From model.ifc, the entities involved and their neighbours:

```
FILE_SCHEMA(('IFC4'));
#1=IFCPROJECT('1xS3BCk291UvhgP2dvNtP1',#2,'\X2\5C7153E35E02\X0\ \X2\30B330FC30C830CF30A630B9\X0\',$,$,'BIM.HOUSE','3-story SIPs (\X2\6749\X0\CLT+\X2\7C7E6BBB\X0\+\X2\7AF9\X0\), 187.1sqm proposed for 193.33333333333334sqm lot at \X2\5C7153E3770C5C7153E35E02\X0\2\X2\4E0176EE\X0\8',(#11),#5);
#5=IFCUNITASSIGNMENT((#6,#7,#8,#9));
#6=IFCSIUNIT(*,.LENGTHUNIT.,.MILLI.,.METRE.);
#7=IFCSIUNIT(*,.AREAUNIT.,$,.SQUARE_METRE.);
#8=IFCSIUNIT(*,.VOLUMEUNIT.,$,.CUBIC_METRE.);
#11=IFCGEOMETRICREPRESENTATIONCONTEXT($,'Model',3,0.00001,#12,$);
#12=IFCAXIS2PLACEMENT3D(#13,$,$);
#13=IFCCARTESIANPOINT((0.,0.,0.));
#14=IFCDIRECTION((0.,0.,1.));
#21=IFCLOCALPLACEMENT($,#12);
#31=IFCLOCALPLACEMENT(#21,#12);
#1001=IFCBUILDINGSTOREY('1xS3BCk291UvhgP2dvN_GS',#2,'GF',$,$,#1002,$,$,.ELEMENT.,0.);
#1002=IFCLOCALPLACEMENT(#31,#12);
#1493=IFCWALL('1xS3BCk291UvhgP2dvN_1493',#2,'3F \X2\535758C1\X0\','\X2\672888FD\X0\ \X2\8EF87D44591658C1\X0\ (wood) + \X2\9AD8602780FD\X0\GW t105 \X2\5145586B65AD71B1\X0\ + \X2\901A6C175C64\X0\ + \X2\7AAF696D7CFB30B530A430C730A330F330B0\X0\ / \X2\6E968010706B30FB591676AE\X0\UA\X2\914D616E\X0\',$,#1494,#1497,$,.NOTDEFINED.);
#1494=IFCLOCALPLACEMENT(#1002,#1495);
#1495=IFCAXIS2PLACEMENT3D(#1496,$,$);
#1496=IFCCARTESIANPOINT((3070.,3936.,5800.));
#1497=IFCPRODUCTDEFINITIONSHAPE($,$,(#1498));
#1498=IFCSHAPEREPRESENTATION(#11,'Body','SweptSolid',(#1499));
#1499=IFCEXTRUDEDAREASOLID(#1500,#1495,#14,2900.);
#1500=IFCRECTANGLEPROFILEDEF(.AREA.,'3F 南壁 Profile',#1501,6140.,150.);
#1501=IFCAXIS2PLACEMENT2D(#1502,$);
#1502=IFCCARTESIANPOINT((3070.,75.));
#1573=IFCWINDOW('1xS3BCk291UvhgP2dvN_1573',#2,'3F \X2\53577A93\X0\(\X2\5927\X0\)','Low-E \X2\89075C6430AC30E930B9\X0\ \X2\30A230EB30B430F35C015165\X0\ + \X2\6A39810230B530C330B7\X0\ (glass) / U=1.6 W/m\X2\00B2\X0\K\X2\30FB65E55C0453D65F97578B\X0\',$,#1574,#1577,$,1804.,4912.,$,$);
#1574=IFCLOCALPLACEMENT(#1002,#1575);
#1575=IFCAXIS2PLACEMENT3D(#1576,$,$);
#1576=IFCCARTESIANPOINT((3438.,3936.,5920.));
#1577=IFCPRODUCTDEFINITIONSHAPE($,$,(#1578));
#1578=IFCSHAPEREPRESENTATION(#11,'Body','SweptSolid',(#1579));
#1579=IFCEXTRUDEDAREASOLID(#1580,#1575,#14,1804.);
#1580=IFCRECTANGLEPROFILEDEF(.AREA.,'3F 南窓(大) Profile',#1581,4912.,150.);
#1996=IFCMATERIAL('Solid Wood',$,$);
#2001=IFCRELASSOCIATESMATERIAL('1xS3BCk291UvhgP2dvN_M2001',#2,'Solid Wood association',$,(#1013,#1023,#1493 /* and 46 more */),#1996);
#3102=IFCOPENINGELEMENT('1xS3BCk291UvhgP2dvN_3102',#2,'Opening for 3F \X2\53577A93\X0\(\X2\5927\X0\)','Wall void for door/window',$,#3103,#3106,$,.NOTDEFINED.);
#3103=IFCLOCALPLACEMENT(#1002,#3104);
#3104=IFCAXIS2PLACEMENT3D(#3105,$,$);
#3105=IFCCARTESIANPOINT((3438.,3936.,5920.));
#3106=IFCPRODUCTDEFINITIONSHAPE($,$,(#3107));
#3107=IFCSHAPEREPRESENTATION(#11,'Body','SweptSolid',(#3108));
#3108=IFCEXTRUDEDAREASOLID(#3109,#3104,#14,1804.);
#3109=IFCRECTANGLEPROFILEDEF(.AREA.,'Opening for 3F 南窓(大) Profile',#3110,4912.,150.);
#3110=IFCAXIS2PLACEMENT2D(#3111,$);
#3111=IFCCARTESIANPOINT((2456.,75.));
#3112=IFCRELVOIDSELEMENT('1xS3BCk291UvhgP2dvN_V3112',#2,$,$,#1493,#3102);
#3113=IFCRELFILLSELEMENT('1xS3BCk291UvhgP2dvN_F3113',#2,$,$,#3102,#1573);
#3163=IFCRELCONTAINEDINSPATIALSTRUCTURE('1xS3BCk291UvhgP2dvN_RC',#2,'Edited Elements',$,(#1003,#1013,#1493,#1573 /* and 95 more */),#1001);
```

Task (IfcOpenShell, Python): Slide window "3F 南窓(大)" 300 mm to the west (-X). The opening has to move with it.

```python
import ifcopenshell
import ifcopenshell.api.geometry
import ifcopenshell.util.placement
import ifcopenshell.util.unit

model = ifcopenshell.open("model.ifc")
unit_scale = ifcopenshell.util.unit.calculate_unit_scale(model)

window = model.by_guid("1xS3BCk291UvhgP2dvN_1573")
opening = window.FillsVoids[0].RelatingOpeningElement
wall = opening.VoidsElements[0].RelatingBuildingElement

wall_matrix = ifcopenshell.util.placement.get_local_placement(wall.ObjectPlacement)
shift = wall_matrix[:3, 0] * -0.3 / unit_scale
before = ifcopenshell.util.placement.get_local_placement(window.ObjectPlacement)[:3, 3].copy()

# The window is not placed relative to its opening, so move both.
for product in (opening, window):
    matrix = ifcopenshell.util.placement.get_local_placement(product.ObjectPlacement)
    matrix[:3, 3] += shift
    ifcopenshell.api.geometry.edit_object_placement(model, product=product, matrix=matrix, is_si=False)

after = ifcopenshell.util.placement.get_local_placement(window.ObjectPlacement)[:3, 3]
print("window moved by", (after - before).round(3) + 0.0)

model.write("model_rev.ifc")
```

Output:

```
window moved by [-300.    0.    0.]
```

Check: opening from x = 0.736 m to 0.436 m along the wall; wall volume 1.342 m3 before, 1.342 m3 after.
